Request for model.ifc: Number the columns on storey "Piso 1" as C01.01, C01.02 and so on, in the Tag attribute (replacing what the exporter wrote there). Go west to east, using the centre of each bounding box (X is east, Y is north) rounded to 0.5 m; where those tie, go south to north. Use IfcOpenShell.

First a look at what the model holds.

```python
import ifcopenshell
import ifcopenshell.util.element
import ifcopenshell.util.placement

model = ifcopenshell.open("model.ifc")
print(model.schema)
storey = next(s for s in model.by_type("IfcBuildingStorey") if s.Name == "Piso 1")
columns = [e for e in ifcopenshell.util.element.get_decomposition(storey) if e.is_a("IfcColumn")]
for e in sorted(columns, key=lambda e: e.id()):
    origin = ifcopenshell.util.placement.get_local_placement(e.ObjectPlacement)[:3, 3]
    print(e.id(), e.Tag, e.Name, origin.round(2) + 0.0, sep=" | ")
```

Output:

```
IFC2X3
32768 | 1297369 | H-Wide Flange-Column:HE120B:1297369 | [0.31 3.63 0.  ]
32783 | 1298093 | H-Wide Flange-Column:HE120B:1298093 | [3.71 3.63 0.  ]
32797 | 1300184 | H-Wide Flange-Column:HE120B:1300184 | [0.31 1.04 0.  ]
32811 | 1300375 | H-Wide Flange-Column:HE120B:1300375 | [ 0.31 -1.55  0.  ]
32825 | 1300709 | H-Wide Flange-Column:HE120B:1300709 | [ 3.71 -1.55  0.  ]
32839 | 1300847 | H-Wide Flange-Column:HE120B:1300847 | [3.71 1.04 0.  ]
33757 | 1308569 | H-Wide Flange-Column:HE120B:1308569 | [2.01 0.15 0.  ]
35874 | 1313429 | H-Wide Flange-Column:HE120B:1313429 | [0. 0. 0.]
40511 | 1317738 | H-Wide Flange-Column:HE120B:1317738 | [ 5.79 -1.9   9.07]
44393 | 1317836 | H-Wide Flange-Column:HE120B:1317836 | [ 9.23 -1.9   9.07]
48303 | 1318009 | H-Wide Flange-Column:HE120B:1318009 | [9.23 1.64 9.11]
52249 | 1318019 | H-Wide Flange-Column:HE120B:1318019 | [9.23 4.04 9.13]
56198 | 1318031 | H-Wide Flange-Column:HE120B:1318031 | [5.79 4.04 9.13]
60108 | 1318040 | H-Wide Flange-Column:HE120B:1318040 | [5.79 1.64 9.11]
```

```python
import ifcopenshell
import ifcopenshell.geom
import ifcopenshell.util.element
import ifcopenshell.util.shape

model = ifcopenshell.open("model.ifc")
settings = ifcopenshell.geom.settings()
settings.set("use-world-coords", True)


def centre(element):
    shape = ifcopenshell.geom.create_shape(settings, element)
    return ifcopenshell.util.shape.get_bbox_centroid(shape.geometry)


storey = next(s for s in model.by_type("IfcBuildingStorey") if s.Name == "Piso 1")
columns = [e for e in ifcopenshell.util.element.get_decomposition(storey) if e.is_a("IfcColumn")]

# Insertion points can sit at a corner or the storey origin, so sort by the geometry (in metres).
centres = {e: centre(e) for e in columns}
columns.sort(key=lambda e: (round(centres[e][0] / 0.5), centres[e][1]))

for i, e in enumerate(columns, start=1):
    number = f"C01.{i:02d}"
    e.Tag = number
    print(e.id(), number)

model.write("model_rev.ifc")
```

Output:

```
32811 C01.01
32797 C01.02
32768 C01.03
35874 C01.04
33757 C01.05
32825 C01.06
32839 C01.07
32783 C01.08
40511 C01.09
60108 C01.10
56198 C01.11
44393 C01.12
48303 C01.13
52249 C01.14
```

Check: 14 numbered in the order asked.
